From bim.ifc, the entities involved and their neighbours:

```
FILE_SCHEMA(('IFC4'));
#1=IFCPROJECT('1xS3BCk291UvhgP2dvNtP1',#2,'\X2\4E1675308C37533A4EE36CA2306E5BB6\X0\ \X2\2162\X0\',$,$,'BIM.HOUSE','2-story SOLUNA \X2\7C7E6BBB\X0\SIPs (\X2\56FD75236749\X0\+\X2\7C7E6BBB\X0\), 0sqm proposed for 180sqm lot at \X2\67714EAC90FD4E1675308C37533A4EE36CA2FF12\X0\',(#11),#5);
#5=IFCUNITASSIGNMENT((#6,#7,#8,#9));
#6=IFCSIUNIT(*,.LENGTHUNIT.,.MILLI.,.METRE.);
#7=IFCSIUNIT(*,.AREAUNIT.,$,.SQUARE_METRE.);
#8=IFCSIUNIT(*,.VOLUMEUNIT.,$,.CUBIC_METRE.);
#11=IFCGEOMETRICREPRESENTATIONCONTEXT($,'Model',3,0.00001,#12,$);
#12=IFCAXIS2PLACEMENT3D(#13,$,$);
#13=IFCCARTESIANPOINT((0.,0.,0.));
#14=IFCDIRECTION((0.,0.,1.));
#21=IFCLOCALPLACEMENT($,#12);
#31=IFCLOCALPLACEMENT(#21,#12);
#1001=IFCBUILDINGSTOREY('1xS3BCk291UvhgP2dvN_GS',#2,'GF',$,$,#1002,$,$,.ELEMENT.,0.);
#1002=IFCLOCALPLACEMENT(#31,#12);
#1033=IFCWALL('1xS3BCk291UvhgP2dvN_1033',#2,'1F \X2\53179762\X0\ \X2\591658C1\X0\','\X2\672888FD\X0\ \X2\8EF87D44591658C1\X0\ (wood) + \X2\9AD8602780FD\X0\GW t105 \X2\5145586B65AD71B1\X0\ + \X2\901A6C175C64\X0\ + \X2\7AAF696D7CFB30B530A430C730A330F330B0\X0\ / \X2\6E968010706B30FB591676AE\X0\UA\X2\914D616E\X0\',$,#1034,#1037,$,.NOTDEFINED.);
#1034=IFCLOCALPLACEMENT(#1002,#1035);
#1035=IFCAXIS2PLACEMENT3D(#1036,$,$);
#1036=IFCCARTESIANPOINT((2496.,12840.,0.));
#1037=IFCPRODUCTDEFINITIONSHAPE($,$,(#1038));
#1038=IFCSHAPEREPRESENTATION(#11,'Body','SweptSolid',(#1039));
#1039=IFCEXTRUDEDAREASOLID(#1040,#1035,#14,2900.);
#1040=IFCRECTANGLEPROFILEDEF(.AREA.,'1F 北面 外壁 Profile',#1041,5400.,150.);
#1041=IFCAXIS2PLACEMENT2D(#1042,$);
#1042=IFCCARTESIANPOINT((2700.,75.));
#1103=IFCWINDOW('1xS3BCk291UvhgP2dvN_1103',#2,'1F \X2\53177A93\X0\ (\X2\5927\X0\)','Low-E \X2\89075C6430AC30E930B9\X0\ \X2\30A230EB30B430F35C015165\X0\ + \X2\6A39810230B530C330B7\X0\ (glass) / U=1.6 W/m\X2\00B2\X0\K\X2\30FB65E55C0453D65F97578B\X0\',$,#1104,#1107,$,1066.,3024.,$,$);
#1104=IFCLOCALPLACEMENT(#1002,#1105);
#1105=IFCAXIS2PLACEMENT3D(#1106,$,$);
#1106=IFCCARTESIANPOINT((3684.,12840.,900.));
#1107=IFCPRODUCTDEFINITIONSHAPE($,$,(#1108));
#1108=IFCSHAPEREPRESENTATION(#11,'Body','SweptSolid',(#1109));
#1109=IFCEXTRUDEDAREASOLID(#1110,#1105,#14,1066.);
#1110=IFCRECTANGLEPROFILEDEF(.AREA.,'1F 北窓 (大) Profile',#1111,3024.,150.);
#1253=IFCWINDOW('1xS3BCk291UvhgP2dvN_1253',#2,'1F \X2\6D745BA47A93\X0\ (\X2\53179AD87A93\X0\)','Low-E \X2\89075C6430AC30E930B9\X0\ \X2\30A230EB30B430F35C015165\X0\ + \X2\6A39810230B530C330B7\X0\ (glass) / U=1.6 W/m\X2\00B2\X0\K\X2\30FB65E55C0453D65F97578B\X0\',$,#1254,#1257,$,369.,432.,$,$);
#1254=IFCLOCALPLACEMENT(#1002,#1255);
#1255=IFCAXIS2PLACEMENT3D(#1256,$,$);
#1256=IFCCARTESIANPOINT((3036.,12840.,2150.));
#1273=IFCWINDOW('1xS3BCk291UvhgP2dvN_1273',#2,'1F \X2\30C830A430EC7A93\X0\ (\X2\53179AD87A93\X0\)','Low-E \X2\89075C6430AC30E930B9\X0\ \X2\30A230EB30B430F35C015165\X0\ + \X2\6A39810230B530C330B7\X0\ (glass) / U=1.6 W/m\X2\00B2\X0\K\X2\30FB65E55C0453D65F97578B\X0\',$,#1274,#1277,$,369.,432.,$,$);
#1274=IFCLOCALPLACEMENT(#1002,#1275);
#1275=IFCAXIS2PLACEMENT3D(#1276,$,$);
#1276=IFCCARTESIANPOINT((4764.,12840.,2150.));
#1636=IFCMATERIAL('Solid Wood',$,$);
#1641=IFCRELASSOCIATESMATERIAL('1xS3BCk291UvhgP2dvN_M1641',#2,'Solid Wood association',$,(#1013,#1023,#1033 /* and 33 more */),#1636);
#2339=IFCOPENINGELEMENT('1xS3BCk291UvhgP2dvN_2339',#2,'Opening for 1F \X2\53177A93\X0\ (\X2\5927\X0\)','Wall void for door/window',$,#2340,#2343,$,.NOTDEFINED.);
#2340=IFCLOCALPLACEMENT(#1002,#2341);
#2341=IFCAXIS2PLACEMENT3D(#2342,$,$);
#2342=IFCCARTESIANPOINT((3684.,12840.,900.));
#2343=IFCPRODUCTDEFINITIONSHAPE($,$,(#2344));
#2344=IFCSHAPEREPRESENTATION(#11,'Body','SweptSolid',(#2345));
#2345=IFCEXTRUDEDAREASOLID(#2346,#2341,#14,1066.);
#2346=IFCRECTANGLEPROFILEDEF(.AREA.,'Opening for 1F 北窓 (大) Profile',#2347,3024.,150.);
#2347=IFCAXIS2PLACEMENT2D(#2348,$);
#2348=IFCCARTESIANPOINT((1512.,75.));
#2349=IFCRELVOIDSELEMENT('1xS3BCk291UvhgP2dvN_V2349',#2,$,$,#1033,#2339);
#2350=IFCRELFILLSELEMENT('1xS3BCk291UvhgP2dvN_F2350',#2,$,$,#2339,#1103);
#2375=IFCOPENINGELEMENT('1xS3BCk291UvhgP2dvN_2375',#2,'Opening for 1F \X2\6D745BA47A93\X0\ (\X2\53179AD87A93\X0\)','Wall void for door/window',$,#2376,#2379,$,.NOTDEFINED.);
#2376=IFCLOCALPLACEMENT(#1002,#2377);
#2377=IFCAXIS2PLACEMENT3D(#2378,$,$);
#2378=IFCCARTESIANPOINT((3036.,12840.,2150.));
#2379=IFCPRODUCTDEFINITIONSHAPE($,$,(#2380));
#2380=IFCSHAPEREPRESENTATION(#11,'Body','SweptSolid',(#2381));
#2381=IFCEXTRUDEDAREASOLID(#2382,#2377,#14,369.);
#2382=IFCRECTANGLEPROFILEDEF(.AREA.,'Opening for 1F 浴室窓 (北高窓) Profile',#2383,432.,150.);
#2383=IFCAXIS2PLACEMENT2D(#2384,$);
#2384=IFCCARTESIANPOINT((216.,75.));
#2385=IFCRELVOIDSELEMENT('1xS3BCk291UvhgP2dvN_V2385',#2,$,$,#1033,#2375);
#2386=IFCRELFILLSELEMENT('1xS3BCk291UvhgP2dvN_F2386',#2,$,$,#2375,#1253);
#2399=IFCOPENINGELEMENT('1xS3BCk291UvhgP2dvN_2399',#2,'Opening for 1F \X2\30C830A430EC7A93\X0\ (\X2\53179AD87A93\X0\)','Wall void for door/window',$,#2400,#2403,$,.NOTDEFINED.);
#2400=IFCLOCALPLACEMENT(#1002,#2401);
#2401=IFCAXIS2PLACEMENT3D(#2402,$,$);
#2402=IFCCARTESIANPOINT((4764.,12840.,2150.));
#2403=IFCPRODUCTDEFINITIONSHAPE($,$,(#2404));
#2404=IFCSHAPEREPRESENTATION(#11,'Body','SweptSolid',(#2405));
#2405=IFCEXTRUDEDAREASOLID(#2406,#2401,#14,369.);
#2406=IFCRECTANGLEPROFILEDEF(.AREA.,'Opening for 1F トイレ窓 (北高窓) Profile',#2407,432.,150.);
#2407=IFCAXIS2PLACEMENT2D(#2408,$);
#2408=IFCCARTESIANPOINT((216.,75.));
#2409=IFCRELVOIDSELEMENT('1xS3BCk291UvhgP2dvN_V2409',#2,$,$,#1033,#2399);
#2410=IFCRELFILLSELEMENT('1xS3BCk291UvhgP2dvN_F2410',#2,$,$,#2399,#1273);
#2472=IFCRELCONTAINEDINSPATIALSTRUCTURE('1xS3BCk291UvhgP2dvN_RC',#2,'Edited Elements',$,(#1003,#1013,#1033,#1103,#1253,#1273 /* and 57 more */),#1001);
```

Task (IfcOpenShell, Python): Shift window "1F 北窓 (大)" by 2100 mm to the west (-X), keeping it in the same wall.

```python
import ifcopenshell
import ifcopenshell.api.geometry
import ifcopenshell.util.placement

model = ifcopenshell.open("bim.ifc")

window = model.by_id(1103)
opening = window.FillsVoids[0].RelatingOpeningElement
wall = opening.VoidsElements[0].RelatingBuildingElement

wall_matrix = ifcopenshell.util.placement.get_local_placement(wall.ObjectPlacement)
shift = wall_matrix[:3, 0] * -2100.0
before = ifcopenshell.util.placement.get_local_placement(window.ObjectPlacement)[:3, 3].copy()

# The window is not placed relative to its opening, so move both.
for product in (opening, window):
    matrix = ifcopenshell.util.placement.get_local_placement(product.ObjectPlacement)
    matrix[:3, 3] += shift
    ifcopenshell.api.geometry.edit_object_placement(model, product=product, matrix=matrix, is_si=False)

after = ifcopenshell.util.placement.get_local_placement(window.ObjectPlacement)[:3, 3]
print("window moved by", (after - before).round(3) + 0.0)

model.write("bim-out.ifc")
```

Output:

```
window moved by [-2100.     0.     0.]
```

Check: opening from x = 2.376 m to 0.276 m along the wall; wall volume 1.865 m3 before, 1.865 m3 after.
